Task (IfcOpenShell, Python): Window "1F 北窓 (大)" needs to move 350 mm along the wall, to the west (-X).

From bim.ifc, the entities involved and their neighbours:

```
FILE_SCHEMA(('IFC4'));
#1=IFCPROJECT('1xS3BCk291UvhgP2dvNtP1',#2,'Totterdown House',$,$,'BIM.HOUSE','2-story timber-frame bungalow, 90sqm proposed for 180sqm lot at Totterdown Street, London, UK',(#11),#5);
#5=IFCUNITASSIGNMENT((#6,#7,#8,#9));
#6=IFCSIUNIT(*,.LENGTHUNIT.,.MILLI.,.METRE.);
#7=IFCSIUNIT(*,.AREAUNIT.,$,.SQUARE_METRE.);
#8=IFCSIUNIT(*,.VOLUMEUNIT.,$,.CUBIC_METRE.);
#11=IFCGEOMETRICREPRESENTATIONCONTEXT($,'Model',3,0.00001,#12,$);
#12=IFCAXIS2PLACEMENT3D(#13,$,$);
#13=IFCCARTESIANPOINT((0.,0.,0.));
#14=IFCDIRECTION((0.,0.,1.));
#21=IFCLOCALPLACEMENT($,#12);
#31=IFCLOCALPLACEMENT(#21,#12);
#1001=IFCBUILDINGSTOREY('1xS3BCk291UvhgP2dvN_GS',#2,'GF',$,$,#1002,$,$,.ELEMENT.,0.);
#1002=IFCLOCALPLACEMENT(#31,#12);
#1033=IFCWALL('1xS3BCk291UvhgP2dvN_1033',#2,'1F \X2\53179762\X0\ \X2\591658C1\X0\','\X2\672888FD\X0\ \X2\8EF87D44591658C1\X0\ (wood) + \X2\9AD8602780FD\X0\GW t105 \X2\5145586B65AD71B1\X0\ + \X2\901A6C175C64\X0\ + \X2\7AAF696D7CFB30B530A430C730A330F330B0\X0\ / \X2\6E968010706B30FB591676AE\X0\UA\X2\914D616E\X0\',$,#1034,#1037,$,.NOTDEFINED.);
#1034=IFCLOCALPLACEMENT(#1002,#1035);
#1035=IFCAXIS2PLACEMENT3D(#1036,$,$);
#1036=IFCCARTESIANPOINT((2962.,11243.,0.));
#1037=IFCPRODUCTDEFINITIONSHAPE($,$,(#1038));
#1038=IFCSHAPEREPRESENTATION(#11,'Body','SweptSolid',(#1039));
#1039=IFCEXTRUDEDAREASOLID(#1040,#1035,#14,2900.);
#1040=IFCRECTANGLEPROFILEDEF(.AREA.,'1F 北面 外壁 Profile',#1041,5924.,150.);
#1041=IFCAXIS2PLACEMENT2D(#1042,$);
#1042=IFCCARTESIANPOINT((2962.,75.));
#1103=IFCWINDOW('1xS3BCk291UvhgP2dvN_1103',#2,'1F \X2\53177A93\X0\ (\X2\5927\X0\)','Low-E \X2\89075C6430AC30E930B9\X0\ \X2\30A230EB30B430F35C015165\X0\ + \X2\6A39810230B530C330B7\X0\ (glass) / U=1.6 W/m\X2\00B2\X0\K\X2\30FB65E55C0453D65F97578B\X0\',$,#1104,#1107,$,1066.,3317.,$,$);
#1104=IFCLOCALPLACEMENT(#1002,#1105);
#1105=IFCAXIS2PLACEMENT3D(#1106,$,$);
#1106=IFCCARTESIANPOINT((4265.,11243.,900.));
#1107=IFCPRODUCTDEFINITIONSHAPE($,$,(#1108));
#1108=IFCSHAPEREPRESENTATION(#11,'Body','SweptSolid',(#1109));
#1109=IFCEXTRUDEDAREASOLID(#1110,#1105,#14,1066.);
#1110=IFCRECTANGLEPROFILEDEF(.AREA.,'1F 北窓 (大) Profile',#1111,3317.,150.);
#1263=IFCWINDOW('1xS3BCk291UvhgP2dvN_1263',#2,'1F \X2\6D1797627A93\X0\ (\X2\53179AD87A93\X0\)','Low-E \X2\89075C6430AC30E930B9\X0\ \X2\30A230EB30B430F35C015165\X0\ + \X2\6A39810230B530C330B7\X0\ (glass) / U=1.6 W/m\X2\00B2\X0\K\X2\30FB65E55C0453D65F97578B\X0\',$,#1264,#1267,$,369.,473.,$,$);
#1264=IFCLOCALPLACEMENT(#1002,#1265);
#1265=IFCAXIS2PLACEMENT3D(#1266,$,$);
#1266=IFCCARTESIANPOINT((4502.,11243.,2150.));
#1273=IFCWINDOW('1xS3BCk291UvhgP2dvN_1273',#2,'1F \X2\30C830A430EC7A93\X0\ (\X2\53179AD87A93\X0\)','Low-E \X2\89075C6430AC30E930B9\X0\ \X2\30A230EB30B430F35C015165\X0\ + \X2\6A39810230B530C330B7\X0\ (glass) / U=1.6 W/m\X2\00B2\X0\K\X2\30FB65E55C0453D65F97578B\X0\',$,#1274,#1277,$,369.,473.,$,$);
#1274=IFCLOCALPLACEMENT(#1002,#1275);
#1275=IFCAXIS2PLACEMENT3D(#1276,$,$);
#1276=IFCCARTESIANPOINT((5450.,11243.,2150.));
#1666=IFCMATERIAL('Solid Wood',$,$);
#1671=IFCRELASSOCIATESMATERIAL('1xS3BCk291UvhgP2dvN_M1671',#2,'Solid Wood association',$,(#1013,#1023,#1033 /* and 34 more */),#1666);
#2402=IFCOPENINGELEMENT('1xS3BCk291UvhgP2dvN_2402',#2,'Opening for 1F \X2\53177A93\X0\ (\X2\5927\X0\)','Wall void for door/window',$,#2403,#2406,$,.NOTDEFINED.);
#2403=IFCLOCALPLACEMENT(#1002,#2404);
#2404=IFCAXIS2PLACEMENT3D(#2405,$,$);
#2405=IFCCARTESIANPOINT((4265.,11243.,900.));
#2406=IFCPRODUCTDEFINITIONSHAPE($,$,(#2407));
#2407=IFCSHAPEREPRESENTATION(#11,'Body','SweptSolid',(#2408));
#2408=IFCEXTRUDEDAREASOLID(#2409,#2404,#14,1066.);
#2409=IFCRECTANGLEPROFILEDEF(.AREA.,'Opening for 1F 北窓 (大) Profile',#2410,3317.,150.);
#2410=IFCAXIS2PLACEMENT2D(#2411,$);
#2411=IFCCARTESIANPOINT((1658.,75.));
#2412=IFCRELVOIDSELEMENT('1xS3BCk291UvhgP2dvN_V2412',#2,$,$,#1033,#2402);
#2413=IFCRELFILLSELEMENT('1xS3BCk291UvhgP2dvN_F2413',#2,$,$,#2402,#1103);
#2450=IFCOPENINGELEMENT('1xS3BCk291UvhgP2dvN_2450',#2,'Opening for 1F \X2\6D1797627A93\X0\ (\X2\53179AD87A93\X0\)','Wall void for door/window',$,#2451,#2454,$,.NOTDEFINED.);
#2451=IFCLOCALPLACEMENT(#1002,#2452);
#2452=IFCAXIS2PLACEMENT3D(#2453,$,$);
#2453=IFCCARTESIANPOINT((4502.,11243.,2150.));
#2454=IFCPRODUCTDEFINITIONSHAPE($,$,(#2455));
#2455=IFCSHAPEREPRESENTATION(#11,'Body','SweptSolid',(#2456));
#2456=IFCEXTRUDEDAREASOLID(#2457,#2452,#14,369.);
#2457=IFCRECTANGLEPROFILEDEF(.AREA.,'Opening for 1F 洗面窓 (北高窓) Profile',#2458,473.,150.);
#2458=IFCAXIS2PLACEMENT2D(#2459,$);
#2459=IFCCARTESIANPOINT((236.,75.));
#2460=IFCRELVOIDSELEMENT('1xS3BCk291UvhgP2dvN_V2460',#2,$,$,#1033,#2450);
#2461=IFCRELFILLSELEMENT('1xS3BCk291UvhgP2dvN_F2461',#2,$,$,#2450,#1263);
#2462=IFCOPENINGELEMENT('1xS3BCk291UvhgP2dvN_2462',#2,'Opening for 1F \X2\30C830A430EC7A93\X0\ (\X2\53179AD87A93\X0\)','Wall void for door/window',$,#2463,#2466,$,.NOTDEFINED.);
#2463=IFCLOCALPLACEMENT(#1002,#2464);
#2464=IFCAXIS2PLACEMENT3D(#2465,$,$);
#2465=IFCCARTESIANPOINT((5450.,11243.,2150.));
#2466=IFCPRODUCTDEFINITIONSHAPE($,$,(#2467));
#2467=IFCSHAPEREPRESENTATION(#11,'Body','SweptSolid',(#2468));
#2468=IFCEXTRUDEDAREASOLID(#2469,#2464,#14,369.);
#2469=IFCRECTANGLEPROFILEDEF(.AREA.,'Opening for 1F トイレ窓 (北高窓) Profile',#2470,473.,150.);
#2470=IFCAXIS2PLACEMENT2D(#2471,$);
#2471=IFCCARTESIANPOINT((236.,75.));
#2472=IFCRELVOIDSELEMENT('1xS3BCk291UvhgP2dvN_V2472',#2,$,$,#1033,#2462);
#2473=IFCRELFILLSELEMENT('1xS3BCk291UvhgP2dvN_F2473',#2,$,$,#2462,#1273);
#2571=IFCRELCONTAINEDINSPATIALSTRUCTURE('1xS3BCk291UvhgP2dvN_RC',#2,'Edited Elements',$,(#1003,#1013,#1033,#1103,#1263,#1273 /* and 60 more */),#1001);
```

```python
import ifcopenshell
import ifcopenshell.api.geometry
import ifcopenshell.util.placement

model = ifcopenshell.open("bim.ifc")

window = model.by_guid("1xS3BCk291UvhgP2dvN_1103")
opening = window.FillsVoids[0].RelatingOpeningElement
wall = opening.VoidsElements[0].RelatingBuildingElement

wall_matrix = ifcopenshell.util.placement.get_local_placement(wall.ObjectPlacement)
shift = wall_matrix[:3, 0] * -350.0
before = ifcopenshell.util.placement.get_local_placement(window.ObjectPlacement)[:3, 3].copy()

# The window is not placed relative to its opening, so move both.
for product in (opening, window):
    matrix = ifcopenshell.util.placement.get_local_placement(product.ObjectPlacement)
    matrix[:3, 3] += shift
    ifcopenshell.api.geometry.edit_object_placement(model, product=product, matrix=matrix, is_si=False)

after = ifcopenshell.util.placement.get_local_placement(window.ObjectPlacement)[:3, 3]
print("window moved by", (after - before).round(3) + 0.0)

model.write("bim_edited.ifc")
```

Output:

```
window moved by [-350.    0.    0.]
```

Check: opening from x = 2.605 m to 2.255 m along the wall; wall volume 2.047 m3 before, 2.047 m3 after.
